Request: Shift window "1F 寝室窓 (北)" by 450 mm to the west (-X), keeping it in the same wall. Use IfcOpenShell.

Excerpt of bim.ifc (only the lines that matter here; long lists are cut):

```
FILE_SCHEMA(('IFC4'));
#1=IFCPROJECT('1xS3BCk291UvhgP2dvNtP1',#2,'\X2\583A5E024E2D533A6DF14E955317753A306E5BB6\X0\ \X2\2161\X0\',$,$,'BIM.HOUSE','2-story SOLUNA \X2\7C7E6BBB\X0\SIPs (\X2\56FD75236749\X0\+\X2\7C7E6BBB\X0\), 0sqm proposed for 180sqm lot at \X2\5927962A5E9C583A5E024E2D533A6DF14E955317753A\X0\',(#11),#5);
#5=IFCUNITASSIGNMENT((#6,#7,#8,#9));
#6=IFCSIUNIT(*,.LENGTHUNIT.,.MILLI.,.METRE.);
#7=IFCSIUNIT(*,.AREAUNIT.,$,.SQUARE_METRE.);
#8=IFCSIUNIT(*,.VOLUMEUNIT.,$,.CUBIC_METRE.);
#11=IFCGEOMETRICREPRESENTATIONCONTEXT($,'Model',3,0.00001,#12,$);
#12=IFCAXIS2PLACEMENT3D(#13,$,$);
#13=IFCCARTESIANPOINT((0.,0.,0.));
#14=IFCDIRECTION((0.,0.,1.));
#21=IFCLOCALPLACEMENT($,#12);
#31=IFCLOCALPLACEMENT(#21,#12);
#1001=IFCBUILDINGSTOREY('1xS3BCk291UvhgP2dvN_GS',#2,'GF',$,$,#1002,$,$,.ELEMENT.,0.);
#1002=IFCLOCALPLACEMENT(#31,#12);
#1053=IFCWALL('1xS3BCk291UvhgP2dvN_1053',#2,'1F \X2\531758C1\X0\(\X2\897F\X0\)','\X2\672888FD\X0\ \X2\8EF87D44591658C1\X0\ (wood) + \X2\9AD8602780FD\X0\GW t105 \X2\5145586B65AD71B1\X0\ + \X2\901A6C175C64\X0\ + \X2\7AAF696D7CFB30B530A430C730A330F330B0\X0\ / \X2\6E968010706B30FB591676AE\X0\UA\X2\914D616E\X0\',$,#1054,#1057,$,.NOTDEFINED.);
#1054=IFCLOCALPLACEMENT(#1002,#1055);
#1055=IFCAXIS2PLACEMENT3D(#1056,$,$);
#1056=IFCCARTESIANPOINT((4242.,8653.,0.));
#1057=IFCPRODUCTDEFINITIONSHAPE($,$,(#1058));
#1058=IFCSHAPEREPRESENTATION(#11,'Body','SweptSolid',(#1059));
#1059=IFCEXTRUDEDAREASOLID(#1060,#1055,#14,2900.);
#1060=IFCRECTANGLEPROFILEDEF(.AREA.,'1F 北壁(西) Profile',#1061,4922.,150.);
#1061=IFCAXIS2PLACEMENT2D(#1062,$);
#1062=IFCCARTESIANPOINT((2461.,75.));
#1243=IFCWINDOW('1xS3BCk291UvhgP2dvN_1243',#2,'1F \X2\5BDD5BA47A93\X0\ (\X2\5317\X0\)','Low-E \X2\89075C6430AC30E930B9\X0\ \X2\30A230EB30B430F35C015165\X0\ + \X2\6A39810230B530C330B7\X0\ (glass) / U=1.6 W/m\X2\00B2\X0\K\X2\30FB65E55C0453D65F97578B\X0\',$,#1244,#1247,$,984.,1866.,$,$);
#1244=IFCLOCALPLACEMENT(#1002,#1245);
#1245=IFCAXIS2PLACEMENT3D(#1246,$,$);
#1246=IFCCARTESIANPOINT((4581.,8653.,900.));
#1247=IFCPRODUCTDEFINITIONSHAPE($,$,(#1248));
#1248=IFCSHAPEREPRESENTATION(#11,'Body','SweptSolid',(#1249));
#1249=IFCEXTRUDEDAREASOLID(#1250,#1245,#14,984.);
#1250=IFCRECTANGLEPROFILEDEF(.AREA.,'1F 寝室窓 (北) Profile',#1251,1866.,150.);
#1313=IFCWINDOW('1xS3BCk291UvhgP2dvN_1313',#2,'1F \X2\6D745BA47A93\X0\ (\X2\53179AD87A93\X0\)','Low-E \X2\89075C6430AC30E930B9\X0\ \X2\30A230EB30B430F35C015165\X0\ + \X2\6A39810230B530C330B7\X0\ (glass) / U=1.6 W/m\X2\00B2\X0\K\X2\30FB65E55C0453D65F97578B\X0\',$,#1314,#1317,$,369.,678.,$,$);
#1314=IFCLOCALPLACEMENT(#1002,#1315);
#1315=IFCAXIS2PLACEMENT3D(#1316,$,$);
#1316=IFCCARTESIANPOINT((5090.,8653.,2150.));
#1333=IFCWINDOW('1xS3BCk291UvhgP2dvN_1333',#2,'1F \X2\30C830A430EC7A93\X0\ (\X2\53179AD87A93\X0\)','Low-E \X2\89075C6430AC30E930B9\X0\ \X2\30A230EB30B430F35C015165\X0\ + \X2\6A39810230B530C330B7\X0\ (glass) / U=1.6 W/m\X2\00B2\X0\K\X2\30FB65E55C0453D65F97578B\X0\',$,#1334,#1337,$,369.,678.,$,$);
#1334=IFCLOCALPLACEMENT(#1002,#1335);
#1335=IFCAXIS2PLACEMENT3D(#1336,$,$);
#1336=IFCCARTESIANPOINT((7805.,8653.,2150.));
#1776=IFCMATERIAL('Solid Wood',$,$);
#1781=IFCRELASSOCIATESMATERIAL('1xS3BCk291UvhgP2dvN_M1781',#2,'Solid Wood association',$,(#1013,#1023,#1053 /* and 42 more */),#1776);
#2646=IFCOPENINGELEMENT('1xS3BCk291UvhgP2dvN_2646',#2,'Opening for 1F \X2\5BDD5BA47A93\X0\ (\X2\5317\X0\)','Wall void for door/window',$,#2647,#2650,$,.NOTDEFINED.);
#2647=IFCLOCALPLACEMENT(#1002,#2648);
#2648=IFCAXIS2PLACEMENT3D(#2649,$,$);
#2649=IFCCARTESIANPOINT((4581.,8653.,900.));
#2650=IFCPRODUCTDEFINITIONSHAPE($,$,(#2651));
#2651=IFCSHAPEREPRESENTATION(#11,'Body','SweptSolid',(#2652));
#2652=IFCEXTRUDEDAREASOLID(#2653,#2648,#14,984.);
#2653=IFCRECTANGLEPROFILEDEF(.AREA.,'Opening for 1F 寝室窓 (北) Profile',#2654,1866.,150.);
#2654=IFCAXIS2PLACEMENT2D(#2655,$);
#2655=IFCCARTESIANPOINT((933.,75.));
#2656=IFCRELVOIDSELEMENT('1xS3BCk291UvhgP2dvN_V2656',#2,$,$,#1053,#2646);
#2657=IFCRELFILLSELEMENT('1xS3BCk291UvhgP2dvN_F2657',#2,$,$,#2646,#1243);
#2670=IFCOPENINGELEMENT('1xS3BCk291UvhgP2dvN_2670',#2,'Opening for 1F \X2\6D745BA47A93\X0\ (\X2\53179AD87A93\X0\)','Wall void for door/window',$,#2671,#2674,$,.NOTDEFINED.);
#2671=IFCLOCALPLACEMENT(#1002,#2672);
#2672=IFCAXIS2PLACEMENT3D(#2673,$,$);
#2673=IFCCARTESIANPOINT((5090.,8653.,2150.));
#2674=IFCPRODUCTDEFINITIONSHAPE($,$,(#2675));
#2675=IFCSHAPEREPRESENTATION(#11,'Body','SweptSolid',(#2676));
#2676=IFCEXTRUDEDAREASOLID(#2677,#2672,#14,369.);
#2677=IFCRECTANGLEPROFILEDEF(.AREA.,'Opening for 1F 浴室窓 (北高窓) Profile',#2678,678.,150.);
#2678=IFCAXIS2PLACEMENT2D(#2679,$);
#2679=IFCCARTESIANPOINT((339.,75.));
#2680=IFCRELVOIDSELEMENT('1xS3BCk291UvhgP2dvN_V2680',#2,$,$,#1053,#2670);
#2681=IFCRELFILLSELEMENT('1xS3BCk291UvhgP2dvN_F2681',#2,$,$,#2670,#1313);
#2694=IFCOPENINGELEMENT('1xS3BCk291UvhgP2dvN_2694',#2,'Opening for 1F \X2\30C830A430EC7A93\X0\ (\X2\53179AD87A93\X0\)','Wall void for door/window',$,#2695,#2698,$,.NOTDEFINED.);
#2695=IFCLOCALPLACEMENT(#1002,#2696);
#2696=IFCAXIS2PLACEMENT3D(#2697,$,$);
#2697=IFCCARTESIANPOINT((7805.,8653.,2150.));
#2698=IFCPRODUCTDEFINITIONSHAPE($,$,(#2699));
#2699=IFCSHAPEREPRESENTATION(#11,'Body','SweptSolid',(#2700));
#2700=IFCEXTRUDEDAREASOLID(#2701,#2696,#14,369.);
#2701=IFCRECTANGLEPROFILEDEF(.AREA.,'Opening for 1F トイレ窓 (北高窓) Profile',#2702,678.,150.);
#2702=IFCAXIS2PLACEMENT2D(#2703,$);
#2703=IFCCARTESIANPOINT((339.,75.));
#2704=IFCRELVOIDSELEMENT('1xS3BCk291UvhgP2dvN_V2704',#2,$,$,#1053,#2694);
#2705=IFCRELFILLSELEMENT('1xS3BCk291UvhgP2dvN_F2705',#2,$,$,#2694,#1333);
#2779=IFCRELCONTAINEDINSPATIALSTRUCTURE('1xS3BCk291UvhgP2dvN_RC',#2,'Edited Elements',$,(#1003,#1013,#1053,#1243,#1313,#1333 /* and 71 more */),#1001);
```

```python
import ifcopenshell
import ifcopenshell.api.geometry
import ifcopenshell.util.placement
import ifcopenshell.util.unit

model = ifcopenshell.open("bim.ifc")
unit_scale = ifcopenshell.util.unit.calculate_unit_scale(model)

window = model.by_guid("1xS3BCk291UvhgP2dvN_1243")
opening = window.FillsVoids[0].RelatingOpeningElement
wall = opening.VoidsElements[0].RelatingBuildingElement

wall_matrix = ifcopenshell.util.placement.get_local_placement(wall.ObjectPlacement)
shift = wall_matrix[:3, 0] * -0.45 / unit_scale
before = ifcopenshell.util.placement.get_local_placement(window.ObjectPlacement)[:3, 3].copy()

# The window is not placed relative to its opening, so move both.
for product in (opening, window):
    matrix = ifcopenshell.util.placement.get_local_placement(product.ObjectPlacement)
    matrix[:3, 3] += shift
    ifcopenshell.api.geometry.edit_object_placement(model, product=product, matrix=matrix, is_si=False)

after = ifcopenshell.util.placement.get_local_placement(window.ObjectPlacement)[:3, 3]
print("window moved by", (after - before).round(3) + 0.0)

model.write("bim_edited.ifc")
```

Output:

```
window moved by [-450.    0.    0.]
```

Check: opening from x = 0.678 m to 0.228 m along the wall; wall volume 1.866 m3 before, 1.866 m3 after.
